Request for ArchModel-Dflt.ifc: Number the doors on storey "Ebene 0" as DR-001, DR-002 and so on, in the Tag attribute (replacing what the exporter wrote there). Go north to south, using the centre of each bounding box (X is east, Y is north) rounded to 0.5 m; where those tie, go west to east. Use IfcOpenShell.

First a look at what the model holds.

```python
import ifcopenshell
import ifcopenshell.util.element
import ifcopenshell.util.placement

model = ifcopenshell.open("ArchModel-Dflt.ifc")
print(model.schema)
storey = next(s for s in model.by_type("IfcBuildingStorey") if s.Name == "Ebene 0")
doors = [e for e in ifcopenshell.util.element.get_decomposition(storey) if e.is_a("IfcDoor")]
for e in sorted(doors, key=lambda e: e.id()):
    origin = ifcopenshell.util.placement.get_local_placement(e.ObjectPlacement)[:3, 3]
    print(e.id(), e.Tag, e.Name, origin.round(2) + 0.0, sep=" | ")
```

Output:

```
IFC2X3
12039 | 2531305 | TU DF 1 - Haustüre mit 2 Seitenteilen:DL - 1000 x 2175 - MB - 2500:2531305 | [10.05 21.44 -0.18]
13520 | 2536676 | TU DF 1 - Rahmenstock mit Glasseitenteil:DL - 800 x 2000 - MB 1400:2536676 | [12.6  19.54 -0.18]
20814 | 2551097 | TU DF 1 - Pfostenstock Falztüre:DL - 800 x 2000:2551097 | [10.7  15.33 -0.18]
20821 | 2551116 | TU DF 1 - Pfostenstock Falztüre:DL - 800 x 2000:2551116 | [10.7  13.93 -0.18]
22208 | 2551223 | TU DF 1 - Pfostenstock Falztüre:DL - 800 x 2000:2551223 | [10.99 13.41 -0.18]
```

```python
import ifcopenshell
import ifcopenshell.geom
import ifcopenshell.util.element
import ifcopenshell.util.shape

model = ifcopenshell.open("ArchModel-Dflt.ifc")
settings = ifcopenshell.geom.settings()
settings.set("use-world-coords", True)


def centre(element):
    shape = ifcopenshell.geom.create_shape(settings, element)
    return ifcopenshell.util.shape.get_bbox_centroid(shape.geometry)


storey = next(s for s in model.by_type("IfcBuildingStorey") if s.Name == "Ebene 0")
doors = [e for e in ifcopenshell.util.element.get_decomposition(storey) if e.is_a("IfcDoor")]

# Insertion points can sit at a corner or the storey origin, so sort by the geometry (in metres).
centres = {e: centre(e) for e in doors}
doors.sort(key=lambda e: (-round(centres[e][1] / 0.5), centres[e][0]))

for i, e in enumerate(doors, start=1):
    number = f"DR-0{i:02d}"
    e.Tag = number
    print(e.id(), number)

model.write("ArchModel-Dflt_v2.ifc")
```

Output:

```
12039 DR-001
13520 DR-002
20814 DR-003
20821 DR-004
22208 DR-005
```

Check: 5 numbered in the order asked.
